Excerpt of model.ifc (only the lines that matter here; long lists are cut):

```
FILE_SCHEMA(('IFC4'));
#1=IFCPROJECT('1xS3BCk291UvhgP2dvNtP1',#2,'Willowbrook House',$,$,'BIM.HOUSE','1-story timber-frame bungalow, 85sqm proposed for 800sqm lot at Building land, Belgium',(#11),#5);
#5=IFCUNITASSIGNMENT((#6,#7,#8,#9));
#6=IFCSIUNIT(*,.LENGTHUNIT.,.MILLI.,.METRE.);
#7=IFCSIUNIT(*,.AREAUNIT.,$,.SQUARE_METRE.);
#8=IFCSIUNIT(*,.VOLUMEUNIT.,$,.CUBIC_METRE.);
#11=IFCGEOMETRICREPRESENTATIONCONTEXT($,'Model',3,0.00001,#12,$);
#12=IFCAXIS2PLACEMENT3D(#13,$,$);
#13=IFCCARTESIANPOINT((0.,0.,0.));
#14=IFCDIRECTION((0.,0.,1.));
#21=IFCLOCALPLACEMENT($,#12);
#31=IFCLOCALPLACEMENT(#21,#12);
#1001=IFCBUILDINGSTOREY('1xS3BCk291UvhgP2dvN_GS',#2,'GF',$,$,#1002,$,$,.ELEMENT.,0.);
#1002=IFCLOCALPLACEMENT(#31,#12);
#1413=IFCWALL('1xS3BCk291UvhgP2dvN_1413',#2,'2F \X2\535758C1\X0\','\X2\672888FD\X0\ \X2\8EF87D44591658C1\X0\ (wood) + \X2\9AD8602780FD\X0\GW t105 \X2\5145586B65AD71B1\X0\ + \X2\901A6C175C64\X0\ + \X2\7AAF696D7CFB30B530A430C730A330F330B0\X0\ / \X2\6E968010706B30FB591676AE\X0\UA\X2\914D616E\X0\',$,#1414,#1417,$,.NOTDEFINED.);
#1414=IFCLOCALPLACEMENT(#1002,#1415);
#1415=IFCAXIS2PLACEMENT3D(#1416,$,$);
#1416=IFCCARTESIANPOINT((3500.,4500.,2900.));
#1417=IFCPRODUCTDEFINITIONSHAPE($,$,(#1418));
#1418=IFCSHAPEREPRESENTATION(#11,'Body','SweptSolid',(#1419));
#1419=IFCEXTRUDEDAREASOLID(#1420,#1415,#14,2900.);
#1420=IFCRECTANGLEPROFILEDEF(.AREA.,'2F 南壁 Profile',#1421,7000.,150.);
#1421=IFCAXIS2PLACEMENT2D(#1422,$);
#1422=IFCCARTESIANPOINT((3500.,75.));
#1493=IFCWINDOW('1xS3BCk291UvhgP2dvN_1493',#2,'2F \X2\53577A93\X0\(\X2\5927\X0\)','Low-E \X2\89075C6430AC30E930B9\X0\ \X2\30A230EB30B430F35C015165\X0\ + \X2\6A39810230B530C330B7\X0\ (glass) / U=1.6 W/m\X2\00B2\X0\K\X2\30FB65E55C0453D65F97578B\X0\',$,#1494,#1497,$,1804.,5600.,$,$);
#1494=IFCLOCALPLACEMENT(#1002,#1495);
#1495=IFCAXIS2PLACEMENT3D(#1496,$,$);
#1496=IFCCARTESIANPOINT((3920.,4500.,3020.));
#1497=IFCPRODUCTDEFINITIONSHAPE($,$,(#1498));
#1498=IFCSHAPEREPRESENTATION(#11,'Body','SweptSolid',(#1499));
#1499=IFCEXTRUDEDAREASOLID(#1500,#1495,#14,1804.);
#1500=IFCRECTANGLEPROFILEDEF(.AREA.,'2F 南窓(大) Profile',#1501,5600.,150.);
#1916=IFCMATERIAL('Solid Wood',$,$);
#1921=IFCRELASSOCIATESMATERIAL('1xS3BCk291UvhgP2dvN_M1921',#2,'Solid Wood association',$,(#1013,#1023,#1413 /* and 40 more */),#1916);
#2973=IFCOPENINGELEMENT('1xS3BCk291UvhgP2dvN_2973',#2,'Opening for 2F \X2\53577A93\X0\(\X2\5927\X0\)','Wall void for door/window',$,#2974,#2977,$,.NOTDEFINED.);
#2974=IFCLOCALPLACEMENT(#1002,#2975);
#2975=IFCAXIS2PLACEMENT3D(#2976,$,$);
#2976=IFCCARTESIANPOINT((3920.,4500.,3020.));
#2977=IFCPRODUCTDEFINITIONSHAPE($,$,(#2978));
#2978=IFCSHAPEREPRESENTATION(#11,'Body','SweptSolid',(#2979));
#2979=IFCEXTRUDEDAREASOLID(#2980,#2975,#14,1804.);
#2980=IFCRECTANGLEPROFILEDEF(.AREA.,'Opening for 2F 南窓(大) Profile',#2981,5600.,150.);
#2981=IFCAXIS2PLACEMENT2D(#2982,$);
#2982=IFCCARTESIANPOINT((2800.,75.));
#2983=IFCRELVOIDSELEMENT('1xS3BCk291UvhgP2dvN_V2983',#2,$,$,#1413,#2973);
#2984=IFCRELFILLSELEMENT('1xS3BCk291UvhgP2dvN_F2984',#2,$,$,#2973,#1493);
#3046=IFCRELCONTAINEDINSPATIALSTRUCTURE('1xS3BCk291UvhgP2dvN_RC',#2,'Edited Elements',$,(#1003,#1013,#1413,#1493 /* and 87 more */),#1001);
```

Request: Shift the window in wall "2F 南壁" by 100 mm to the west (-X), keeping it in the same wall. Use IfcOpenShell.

```python
import ifcopenshell
import ifcopenshell.api.geometry
import ifcopenshell.util.placement
import ifcopenshell.util.unit

model = ifcopenshell.open("model.ifc")
unit_scale = ifcopenshell.util.unit.calculate_unit_scale(model)

window = model.by_guid("1xS3BCk291UvhgP2dvN_1493")
opening = window.FillsVoids[0].RelatingOpeningElement
wall = opening.VoidsElements[0].RelatingBuildingElement

wall_matrix = ifcopenshell.util.placement.get_local_placement(wall.ObjectPlacement)
shift = wall_matrix[:3, 0] * -0.1 / unit_scale
before = ifcopenshell.util.placement.get_local_placement(window.ObjectPlacement)[:3, 3].copy()

# The window is not placed relative to its opening, so move both.
for product in (opening, window):
    matrix = ifcopenshell.util.placement.get_local_placement(product.ObjectPlacement)
    matrix[:3, 3] += shift
    ifcopenshell.api.geometry.edit_object_placement(model, product=product, matrix=matrix, is_si=False)

after = ifcopenshell.util.placement.get_local_placement(window.ObjectPlacement)[:3, 3]
print("window moved by", (after - before).round(3) + 0.0)

model.write("model_edited.ifc")
```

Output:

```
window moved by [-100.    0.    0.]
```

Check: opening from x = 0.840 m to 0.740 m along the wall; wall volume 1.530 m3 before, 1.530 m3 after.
